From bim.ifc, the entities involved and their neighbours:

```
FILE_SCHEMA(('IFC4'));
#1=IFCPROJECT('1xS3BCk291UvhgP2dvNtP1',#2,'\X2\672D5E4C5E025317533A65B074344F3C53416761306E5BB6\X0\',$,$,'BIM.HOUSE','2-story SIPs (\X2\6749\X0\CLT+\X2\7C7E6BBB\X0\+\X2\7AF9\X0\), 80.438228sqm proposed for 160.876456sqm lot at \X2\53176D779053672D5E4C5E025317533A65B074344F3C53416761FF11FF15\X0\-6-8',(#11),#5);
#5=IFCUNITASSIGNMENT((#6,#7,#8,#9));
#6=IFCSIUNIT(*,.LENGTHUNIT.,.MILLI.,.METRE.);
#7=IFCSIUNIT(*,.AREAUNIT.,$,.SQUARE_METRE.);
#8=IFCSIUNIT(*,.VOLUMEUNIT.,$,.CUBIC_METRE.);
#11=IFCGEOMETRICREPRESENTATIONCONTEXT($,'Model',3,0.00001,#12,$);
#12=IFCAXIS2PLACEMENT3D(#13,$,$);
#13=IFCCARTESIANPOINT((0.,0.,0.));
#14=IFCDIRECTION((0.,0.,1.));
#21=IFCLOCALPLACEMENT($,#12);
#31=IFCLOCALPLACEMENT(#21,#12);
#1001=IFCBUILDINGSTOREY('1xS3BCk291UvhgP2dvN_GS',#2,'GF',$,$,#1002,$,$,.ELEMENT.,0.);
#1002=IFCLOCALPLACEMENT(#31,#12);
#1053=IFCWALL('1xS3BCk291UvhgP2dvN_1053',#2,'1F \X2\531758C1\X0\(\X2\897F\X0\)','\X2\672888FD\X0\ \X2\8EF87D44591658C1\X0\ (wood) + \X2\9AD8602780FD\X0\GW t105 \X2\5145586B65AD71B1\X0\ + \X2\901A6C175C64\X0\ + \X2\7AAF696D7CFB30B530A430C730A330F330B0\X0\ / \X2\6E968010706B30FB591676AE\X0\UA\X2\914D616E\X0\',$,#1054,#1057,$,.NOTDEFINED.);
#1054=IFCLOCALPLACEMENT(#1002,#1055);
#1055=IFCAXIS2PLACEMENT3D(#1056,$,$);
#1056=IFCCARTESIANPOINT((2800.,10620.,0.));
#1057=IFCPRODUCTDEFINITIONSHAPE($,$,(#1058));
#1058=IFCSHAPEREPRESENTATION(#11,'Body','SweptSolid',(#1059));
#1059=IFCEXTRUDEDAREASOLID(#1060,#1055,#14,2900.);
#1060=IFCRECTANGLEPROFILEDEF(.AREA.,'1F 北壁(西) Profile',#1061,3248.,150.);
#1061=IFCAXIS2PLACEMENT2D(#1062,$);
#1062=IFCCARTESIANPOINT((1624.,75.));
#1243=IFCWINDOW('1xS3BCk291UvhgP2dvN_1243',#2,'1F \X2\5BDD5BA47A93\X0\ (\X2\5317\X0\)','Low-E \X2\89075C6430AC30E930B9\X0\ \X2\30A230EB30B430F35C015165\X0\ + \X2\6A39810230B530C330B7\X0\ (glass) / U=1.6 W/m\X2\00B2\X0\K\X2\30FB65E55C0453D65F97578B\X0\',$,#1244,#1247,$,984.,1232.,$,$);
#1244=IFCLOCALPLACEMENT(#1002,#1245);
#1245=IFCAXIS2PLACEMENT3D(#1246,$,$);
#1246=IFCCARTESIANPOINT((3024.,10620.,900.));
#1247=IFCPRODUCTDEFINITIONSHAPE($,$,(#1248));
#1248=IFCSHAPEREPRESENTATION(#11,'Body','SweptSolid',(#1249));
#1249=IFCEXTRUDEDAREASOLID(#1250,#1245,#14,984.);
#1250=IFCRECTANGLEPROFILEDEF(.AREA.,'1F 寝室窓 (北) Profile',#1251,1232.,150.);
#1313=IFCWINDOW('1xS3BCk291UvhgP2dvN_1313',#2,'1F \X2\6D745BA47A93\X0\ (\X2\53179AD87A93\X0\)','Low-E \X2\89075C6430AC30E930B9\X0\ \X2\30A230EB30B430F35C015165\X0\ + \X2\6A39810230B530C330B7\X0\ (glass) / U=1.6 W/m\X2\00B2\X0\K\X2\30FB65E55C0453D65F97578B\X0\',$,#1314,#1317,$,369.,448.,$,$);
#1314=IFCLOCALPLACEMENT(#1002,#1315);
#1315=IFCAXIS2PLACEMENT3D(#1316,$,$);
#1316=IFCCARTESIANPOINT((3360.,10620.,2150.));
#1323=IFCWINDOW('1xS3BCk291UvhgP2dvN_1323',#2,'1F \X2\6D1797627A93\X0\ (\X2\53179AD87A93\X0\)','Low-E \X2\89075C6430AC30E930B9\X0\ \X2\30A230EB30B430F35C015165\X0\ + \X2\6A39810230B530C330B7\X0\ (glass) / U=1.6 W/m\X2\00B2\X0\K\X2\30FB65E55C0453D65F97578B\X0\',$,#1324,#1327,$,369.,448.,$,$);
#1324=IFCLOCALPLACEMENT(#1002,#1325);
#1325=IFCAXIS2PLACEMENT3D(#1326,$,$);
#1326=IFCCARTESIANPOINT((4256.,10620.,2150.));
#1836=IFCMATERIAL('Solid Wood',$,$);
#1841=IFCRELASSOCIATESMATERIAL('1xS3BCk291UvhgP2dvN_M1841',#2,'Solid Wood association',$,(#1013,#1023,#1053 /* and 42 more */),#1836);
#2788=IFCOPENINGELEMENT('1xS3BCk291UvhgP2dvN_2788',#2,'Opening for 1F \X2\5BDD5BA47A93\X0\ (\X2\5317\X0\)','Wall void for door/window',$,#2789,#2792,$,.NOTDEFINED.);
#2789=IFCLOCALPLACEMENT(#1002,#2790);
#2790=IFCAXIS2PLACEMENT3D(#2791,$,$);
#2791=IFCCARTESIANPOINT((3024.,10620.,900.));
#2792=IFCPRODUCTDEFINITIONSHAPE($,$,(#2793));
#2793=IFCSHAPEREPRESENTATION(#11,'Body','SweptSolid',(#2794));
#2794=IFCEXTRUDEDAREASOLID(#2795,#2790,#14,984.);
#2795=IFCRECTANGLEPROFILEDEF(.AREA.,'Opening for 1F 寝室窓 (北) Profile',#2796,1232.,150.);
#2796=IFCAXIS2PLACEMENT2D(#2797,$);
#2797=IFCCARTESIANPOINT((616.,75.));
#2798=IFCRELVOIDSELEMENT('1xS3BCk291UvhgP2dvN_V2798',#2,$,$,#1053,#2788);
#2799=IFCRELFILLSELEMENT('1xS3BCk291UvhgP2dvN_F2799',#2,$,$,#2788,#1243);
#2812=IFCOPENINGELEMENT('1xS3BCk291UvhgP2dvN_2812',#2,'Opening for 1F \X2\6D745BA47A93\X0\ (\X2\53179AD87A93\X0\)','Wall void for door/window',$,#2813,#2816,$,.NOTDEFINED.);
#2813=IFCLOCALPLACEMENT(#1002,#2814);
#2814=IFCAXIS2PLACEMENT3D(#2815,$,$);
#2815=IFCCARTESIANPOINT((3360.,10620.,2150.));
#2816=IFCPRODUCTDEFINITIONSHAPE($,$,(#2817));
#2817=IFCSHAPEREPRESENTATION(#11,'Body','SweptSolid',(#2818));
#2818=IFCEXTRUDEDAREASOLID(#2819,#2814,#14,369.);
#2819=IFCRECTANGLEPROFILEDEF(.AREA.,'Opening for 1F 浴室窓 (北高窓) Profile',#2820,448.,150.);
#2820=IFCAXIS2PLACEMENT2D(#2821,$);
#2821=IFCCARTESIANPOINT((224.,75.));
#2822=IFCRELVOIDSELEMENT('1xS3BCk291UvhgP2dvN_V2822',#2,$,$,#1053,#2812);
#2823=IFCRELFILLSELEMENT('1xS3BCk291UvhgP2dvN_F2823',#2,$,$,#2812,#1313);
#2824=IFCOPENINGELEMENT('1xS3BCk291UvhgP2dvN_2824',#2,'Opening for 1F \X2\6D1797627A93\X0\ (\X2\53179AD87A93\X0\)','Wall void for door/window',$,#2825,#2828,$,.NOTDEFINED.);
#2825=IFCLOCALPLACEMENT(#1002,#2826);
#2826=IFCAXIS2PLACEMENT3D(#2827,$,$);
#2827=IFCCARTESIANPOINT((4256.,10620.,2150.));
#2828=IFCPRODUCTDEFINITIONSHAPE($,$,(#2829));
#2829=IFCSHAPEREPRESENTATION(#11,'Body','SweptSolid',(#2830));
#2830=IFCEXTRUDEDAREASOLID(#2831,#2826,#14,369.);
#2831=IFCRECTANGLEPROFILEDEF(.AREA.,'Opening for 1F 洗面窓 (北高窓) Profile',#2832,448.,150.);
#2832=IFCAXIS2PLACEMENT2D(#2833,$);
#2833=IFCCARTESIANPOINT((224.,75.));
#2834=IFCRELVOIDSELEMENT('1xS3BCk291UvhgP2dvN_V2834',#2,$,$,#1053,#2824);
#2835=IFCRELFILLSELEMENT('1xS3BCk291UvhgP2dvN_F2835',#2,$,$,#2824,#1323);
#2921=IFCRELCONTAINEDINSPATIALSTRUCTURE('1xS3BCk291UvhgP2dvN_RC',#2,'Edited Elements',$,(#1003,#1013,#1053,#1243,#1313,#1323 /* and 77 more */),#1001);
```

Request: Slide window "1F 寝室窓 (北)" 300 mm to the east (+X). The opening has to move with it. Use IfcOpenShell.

```python
import ifcopenshell
import ifcopenshell.api.geometry
import ifcopenshell.util.placement
import ifcopenshell.util.unit

model = ifcopenshell.open("bim.ifc")
unit_scale = ifcopenshell.util.unit.calculate_unit_scale(model)

window = model.by_guid("1xS3BCk291UvhgP2dvN_1243")
opening = window.FillsVoids[0].RelatingOpeningElement
wall = opening.VoidsElements[0].RelatingBuildingElement

wall_matrix = ifcopenshell.util.placement.get_local_placement(wall.ObjectPlacement)
shift = wall_matrix[:3, 0] * 0.3 / unit_scale
before = ifcopenshell.util.placement.get_local_placement(window.ObjectPlacement)[:3, 3].copy()

# The window is not placed relative to its opening, so move both.
for product in (opening, window):
    matrix = ifcopenshell.util.placement.get_local_placement(product.ObjectPlacement)
    matrix[:3, 3] += shift
    ifcopenshell.api.geometry.edit_object_placement(model, product=product, matrix=matrix, is_si=False)

after = ifcopenshell.util.placement.get_local_placement(window.ObjectPlacement)[:3, 3]
print("window moved by", (after - before).round(3) + 0.0)

model.write("bim-out.ifc")
```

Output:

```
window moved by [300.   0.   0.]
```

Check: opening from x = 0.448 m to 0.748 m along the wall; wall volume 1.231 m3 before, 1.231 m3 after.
